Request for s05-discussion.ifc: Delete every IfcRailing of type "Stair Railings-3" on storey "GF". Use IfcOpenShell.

First a look at what the model holds.

```python
import ifcopenshell
import ifcopenshell.util.element

model = ifcopenshell.open("s05-discussion.ifc")
print(model.schema)
storey = next(s for s in model.by_type("IfcBuildingStorey") if s.Name == "GF")
railings = [e for e in ifcopenshell.util.element.get_decomposition(storey) if e.is_a("IfcRailing")]
seen = {}
for e in railings:
    element_type = ifcopenshell.util.element.get_type(e)
    name = element_type.Name if element_type not in (None, e) else None
    seen[name] = seen.get(name, 0) + 1
for name, count in sorted(seen.items(), key=str):
    print(count, "x", name)
```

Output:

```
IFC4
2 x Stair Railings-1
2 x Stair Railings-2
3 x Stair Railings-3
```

```python
import ifcopenshell
import ifcopenshell.api.root
import ifcopenshell.util.element

model = ifcopenshell.open("s05-discussion.ifc")

storey = next(s for s in model.by_type("IfcBuildingStorey") if s.Name == "GF")
railings = [e for e in ifcopenshell.util.element.get_decomposition(storey) if e.is_a("IfcRailing")]
targets = [e for e in railings if (t := ifcopenshell.util.element.get_type(e)) not in (None, e) and t.Name == "Stair Railings-3"]

for e in targets:
    ifcopenshell.api.root.remove_product(model, product=e)
print(len(targets), "removed")

model.write("s05-discussion_v2.ifc")
```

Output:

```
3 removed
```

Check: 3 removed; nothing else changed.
